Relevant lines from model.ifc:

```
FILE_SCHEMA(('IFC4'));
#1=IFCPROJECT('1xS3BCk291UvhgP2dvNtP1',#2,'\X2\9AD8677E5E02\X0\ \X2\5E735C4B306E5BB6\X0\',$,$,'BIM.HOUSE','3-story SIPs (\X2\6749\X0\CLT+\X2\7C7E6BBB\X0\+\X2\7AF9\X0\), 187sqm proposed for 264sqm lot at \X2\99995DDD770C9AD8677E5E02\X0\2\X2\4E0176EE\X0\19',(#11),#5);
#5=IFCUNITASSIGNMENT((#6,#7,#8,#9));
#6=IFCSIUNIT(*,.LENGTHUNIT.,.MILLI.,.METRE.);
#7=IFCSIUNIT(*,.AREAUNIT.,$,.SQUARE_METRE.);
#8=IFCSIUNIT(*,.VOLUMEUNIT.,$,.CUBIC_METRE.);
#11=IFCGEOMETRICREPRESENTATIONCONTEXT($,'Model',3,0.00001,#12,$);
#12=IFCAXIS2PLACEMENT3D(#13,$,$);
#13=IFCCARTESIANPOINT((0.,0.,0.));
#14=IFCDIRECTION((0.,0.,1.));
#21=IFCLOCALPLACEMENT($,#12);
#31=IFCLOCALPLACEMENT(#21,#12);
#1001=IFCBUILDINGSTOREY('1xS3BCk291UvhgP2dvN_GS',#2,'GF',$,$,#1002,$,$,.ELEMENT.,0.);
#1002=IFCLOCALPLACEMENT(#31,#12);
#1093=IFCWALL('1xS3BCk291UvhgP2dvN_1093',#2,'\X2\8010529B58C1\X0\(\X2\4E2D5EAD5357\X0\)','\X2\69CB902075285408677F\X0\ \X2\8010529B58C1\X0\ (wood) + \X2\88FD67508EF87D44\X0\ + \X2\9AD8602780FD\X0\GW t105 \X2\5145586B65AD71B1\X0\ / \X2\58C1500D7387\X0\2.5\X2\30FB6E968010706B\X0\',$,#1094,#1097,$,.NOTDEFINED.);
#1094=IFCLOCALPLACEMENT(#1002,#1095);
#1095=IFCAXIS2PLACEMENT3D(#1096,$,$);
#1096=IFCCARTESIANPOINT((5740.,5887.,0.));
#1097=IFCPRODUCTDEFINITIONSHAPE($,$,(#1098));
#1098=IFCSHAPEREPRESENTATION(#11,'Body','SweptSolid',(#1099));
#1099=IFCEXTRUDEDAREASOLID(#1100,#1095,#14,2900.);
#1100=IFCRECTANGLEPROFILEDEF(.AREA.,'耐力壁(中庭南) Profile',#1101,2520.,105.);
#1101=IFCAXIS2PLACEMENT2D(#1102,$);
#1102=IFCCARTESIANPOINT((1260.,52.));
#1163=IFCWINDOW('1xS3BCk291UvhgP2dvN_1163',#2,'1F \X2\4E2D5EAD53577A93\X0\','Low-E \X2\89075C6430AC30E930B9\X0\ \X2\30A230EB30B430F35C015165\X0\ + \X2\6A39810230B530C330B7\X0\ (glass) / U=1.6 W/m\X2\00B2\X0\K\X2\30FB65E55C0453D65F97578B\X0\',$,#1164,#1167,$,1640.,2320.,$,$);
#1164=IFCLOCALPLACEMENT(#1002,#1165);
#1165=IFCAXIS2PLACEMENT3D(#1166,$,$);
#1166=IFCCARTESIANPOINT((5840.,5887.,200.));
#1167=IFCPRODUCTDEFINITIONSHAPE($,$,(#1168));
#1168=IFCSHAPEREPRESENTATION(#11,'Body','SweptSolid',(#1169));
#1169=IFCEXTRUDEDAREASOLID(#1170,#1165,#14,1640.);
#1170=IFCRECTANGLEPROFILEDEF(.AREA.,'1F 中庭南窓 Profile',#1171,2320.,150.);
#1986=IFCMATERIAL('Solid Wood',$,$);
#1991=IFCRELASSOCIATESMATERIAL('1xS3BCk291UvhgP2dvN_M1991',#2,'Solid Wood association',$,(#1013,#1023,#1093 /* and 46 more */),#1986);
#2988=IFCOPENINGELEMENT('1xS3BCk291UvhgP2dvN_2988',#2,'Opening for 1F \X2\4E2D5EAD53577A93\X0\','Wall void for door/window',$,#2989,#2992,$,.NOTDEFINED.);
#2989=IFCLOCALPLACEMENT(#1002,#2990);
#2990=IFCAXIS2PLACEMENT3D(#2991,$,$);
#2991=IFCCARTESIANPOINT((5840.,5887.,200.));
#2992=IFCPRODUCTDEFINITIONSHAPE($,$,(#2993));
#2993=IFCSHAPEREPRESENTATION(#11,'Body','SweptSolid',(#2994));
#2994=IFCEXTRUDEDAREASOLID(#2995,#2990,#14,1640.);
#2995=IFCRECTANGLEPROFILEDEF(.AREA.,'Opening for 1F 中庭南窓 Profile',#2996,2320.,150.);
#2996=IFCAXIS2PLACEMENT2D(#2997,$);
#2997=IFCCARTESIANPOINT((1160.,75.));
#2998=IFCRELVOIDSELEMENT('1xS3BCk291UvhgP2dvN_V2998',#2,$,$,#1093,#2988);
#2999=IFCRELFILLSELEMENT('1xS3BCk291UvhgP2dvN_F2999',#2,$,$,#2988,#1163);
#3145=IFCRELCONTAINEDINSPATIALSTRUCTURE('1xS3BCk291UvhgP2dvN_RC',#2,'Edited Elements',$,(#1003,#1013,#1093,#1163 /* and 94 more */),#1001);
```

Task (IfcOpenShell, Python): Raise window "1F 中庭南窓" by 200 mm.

```python
import numpy as np
import ifcopenshell
import ifcopenshell.api.geometry
import ifcopenshell.util.placement
import ifcopenshell.util.unit

model = ifcopenshell.open("model.ifc")
unit_scale = ifcopenshell.util.unit.calculate_unit_scale(model)

window = model.by_id(1163)
opening = window.FillsVoids[0].RelatingOpeningElement
dz = 0.2 / unit_scale

shift = np.array([0.0, 0.0, dz])
# The window is not placed relative to its opening, so move both.
for product in (opening, window):
    matrix = ifcopenshell.util.placement.get_local_placement(product.ObjectPlacement)
    matrix[:3, 3] += shift
    ifcopenshell.api.geometry.edit_object_placement(model, product=product, matrix=matrix, is_si=False)

print(f"moved by {dz * unit_scale:+.3f} m")

model.write("model_rev.ifc")
```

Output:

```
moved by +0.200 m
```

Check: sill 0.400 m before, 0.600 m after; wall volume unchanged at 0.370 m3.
